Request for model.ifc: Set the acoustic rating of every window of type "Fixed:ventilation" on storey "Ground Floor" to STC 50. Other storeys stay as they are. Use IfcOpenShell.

First a look at what the model holds.

```python
import ifcopenshell
import ifcopenshell.util.element

model = ifcopenshell.open("model.ifc")
print(model.schema)
storey = next(s for s in model.by_type("IfcBuildingStorey") if s.Name == "Ground Floor")
windows = [e for e in ifcopenshell.util.element.get_decomposition(storey) if e.is_a("IfcWindow")]
seen = {}
for e in windows:
    element_type = ifcopenshell.util.element.get_type(e)
    key = (element_type.Name if element_type != e and element_type else None, ifcopenshell.util.element.get_pset(e, "Pset_WindowCommon", "AcousticRating"))
    seen[key] = seen.get(key, 0) + 1
for (name, value), count in sorted(seen.items(), key=str):
    print(count, "x", name, "|", value)
```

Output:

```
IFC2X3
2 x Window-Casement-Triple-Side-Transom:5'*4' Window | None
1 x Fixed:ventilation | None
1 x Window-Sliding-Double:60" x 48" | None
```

```python
import ifcopenshell
import ifcopenshell.api.pset
import ifcopenshell.util.element

model = ifcopenshell.open("model.ifc")

storey = next(s for s in model.by_type("IfcBuildingStorey") if s.Name == "Ground Floor")
windows = [e for e in ifcopenshell.util.element.get_decomposition(storey) if e.is_a("IfcWindow")]

count = 0
for e in windows:
    element_type = ifcopenshell.util.element.get_type(e)
    if element_type in (None, e) or element_type.Name != "Fixed:ventilation":
        continue
    # add_pset returns the element's existing set when there is one.
    pset = ifcopenshell.api.pset.add_pset(model, product=e, name="Pset_WindowCommon")
    ifcopenshell.api.pset.edit_pset(model, pset=pset, properties={"AcousticRating": "STC 50"})
    count += 1

print(count, "windows updated")

model.write("model_v2.ifc")
```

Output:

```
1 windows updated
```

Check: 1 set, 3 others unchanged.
